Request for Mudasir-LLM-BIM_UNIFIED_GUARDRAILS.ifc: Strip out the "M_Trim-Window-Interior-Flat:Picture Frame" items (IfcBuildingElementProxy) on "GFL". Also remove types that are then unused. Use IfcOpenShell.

First a look at what the model holds.

```python
import ifcopenshell
import ifcopenshell.util.element

model = ifcopenshell.open("Mudasir-LLM-BIM_UNIFIED_GUARDRAILS.ifc")
print(model.schema)
storey = next(s for s in model.by_type("IfcBuildingStorey") if s.Name == "GFL")
proxies = [e for e in ifcopenshell.util.element.get_decomposition(storey) if e.is_a("IfcBuildingElementProxy")]
seen = {}
for e in proxies:
    element_type = ifcopenshell.util.element.get_type(e)
    name = element_type.Name if element_type not in (None, e) else None
    seen[name] = seen.get(name, 0) + 1
for name, count in sorted(seen.items(), key=str):
    print(count, "x", name)
```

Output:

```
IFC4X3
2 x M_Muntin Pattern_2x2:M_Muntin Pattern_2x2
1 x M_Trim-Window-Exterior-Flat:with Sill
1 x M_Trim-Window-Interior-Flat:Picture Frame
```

```python
import ifcopenshell
import ifcopenshell.api.root
import ifcopenshell.util.element

model = ifcopenshell.open("Mudasir-LLM-BIM_UNIFIED_GUARDRAILS.ifc")

storey = next(s for s in model.by_type("IfcBuildingStorey") if s.Name == "GFL")
proxies = [e for e in ifcopenshell.util.element.get_decomposition(storey) if e.is_a("IfcBuildingElementProxy")]
targets = [e for e in proxies if (t := ifcopenshell.util.element.get_type(e)) not in (None, e) and t.Name == "M_Trim-Window-Interior-Flat:Picture Frame"]
types = {ifcopenshell.util.element.get_type(e) for e in targets} - {None, *targets}

for e in targets:
    ifcopenshell.api.root.remove_product(model, product=e)
print(len(targets), "removed")

unused = [t for t in types if not ifcopenshell.util.element.get_types(t)]
for t in unused:
    ifcopenshell.api.root.remove_product(model, product=t)
print(len(unused), "unused types removed")

model.write("Mudasir-LLM-BIM_UNIFIED_GUARDRAILS_v2.ifc")
```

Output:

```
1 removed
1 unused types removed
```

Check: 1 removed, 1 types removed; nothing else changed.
